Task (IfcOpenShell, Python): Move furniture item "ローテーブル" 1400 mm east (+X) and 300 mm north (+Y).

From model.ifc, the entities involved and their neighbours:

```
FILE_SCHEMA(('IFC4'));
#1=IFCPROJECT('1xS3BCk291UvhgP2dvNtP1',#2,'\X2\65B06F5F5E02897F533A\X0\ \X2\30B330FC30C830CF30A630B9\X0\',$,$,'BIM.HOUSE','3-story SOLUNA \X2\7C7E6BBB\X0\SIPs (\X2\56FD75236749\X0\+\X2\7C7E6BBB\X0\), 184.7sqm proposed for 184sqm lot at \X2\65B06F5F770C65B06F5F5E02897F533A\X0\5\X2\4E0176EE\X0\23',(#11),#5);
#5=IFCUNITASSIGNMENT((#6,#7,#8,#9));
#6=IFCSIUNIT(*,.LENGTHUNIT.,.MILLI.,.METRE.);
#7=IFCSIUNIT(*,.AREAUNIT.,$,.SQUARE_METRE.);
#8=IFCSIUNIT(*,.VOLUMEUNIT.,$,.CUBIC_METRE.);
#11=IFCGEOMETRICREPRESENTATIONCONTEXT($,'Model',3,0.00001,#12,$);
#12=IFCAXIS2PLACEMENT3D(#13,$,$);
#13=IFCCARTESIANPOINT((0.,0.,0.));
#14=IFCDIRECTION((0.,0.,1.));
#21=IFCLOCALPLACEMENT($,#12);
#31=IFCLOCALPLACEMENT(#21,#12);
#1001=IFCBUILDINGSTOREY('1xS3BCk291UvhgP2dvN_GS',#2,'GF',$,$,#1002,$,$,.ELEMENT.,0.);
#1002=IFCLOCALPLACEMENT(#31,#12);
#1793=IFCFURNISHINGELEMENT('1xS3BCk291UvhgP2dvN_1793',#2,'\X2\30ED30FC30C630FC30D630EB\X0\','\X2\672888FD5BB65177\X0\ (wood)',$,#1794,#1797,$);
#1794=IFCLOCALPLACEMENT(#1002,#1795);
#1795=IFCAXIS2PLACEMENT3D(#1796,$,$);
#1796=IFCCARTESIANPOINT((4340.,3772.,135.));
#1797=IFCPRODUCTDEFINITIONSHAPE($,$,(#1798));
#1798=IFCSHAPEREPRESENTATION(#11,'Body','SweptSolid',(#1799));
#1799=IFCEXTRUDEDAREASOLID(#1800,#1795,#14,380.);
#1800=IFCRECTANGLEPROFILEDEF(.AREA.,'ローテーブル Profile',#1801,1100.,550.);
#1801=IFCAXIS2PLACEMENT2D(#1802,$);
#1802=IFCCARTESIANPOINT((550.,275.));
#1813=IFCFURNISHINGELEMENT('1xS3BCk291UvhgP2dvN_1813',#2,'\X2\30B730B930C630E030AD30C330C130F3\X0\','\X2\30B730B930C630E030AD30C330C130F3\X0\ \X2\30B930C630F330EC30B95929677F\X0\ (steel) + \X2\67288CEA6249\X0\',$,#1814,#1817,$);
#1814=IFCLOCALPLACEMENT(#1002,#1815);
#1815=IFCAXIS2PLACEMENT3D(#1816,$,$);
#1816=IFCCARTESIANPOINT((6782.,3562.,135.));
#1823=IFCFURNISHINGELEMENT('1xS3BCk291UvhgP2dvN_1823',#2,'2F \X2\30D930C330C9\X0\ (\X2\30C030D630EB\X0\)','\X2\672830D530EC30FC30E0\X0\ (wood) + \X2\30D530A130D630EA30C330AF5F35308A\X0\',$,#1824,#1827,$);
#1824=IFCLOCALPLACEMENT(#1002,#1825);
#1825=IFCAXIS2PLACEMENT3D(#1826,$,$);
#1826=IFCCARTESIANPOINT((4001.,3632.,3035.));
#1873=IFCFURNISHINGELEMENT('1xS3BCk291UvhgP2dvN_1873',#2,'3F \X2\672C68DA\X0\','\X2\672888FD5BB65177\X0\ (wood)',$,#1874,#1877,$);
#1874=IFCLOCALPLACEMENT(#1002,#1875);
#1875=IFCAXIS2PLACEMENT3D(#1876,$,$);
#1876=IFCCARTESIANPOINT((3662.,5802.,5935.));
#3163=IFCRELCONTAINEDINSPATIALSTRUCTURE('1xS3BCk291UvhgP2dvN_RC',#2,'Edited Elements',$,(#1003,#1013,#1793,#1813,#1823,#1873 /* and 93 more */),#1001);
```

```python
import ifcopenshell
import ifcopenshell.api.geometry
import ifcopenshell.util.placement
import ifcopenshell.util.unit

model = ifcopenshell.open("model.ifc")
unit_scale = ifcopenshell.util.unit.calculate_unit_scale(model)

item = model.by_guid("1xS3BCk291UvhgP2dvN_1793")
matrix = ifcopenshell.util.placement.get_local_placement(item.ObjectPlacement)
matrix[0, 3] += 1.4 / unit_scale
matrix[1, 3] += 0.3 / unit_scale
ifcopenshell.api.geometry.edit_object_placement(model, product=item, matrix=matrix, is_si=False)

print(ifcopenshell.util.placement.get_local_placement(item.ObjectPlacement).round(3) + 0.0)

model.write("model_v2.ifc")
```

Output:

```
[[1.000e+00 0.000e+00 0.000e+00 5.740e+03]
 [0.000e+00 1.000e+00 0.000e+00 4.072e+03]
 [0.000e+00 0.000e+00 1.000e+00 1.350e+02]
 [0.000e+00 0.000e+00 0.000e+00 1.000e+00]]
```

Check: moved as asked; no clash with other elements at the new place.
